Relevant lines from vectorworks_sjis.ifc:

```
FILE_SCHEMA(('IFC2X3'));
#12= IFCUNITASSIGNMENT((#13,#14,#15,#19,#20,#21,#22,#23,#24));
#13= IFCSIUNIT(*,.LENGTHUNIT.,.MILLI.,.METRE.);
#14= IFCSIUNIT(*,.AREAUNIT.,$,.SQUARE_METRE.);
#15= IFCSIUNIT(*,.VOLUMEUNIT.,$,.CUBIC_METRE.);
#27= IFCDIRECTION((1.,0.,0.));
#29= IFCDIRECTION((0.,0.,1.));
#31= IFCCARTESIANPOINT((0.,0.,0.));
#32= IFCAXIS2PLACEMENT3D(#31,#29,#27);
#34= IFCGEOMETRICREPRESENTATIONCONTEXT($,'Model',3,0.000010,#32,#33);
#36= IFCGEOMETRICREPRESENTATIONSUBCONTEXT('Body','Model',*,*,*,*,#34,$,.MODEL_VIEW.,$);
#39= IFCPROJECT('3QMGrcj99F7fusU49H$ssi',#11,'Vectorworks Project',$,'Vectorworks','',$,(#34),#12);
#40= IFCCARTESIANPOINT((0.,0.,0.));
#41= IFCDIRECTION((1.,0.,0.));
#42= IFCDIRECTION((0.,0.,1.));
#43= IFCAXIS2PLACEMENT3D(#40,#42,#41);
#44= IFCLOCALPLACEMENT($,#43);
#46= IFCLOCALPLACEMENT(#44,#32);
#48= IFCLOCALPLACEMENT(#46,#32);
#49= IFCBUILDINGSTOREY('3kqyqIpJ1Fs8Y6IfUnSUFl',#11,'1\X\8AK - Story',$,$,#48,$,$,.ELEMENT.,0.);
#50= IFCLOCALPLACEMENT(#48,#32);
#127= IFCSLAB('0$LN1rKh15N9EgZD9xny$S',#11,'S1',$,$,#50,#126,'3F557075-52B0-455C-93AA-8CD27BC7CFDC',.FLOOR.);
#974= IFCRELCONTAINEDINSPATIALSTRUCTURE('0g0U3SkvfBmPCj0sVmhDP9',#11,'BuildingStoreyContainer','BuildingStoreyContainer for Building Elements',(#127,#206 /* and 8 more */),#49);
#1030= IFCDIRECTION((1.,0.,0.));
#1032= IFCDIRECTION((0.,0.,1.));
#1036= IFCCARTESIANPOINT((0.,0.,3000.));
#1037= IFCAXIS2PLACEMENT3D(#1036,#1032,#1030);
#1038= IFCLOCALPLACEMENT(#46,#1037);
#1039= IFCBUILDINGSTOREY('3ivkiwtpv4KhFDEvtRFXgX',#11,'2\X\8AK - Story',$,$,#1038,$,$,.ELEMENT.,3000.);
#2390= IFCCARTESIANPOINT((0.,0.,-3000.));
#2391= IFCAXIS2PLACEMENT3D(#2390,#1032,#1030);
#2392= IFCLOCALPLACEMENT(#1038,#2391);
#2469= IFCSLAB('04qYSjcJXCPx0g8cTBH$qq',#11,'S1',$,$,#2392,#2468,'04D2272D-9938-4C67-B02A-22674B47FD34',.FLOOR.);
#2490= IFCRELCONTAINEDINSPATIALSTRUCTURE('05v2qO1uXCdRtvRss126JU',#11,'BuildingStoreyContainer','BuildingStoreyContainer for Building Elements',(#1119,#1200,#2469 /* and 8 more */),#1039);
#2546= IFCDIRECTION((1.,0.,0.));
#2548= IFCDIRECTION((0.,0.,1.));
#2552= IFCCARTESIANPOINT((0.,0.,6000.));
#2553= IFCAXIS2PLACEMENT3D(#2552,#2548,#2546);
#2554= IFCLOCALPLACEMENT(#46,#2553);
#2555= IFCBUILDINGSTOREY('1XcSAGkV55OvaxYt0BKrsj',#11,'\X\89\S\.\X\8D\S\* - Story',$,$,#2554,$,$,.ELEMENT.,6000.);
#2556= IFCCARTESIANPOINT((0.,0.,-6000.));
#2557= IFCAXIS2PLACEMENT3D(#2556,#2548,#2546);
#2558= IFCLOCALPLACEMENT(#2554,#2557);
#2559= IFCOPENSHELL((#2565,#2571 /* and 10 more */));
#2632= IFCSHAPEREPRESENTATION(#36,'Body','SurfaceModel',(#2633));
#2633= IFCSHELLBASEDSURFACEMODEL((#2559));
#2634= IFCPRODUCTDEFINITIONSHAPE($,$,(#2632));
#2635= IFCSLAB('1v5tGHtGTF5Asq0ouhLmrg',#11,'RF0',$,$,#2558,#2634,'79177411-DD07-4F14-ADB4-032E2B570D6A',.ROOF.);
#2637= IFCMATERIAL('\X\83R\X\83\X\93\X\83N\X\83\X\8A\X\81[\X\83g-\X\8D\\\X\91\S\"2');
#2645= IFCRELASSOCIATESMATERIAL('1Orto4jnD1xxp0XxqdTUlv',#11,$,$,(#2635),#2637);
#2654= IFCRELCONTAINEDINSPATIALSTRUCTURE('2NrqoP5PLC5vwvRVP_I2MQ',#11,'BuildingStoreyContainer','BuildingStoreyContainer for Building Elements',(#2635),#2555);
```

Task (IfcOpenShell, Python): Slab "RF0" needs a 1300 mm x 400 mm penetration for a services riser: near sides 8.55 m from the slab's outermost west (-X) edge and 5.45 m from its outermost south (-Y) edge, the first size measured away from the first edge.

```python
import numpy as np
import ifcopenshell
import ifcopenshell.api.feature
import ifcopenshell.api.geometry
import ifcopenshell.api.root
import ifcopenshell.geom
import ifcopenshell.util.placement
import ifcopenshell.util.representation
import ifcopenshell.util.shape
import ifcopenshell.util.unit

model = ifcopenshell.open("vectorworks_sjis.ifc")
unit_scale = ifcopenshell.util.unit.calculate_unit_scale(model)
settings = ifcopenshell.geom.settings()


def volume(element):
    """Net volume in cubic metres, openings subtracted."""
    shape = ifcopenshell.geom.create_shape(settings, element)
    return ifcopenshell.util.shape.get_volume(shape.geometry)


slab = model.by_guid("1v5tGHtGTF5Asq0ouhLmrg")
before = volume(slab)

# Extent in the slab's own axes, in metres. The edges named are its -X and -Y sides.
slab_shape = ifcopenshell.geom.create_shape(settings, slab)
vertices = ifcopenshell.util.shape.get_vertices(slab_shape.geometry)
x_min, y_min, bottom = vertices.min(axis=0)
top = vertices[:, 2].max()

opening = ifcopenshell.api.root.create_entity(model, ifc_class="IfcOpeningElement", name="Services riser opening")
context = ifcopenshell.util.representation.get_context(model, "Model", "Body", "MODEL_VIEW")
width, depth = 1.3, 0.4
outline = [(0.0, 0.0), (width, 0.0), (width, depth), (0.0, depth), (0.0, 0.0)]
# Overshoot both faces by 50 mm so the cut is clean.
shape = ifcopenshell.api.geometry.add_slab_representation(
    model, context=context, depth=top - bottom + 0.1, polyline=outline
)
ifcopenshell.api.geometry.assign_representation(model, product=opening, representation=shape)

matrix = ifcopenshell.util.placement.get_local_placement(slab.ObjectPlacement)
matrix[:, 3] = matrix @ np.append(np.array([x_min + 8.55, y_min + 5.45, bottom - 0.05]) / unit_scale, 1.0)
ifcopenshell.api.geometry.edit_object_placement(model, product=opening, matrix=matrix, is_si=False)
ifcopenshell.api.feature.add_feature(model, feature=opening, element=slab)

after = volume(slab)

print(f"slab volume {before:.3f} -> {after:.3f} m3")

model.write("vectorworks_sjis_edited.ifc")
```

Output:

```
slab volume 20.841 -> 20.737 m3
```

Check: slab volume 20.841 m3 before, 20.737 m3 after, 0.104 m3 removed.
